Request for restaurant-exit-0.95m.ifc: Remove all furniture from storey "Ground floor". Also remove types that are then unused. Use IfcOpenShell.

First a look at what the model holds.

```python
import ifcopenshell
import ifcopenshell.util.element

model = ifcopenshell.open("restaurant-exit-0.95m.ifc")
print(model.schema)
storey = next(s for s in model.by_type("IfcBuildingStorey") if s.Name == "Ground floor")
furniture = [e for e in ifcopenshell.util.element.get_decomposition(storey) if e.is_a("IfcFurnishingElement")]
seen = {}
for e in furniture:
    element_type = ifcopenshell.util.element.get_type(e)
    name = element_type.Name if element_type not in (None, e) else None
    seen[name] = seen.get(name, 0) + 1
for name, count in sorted(seen.items(), key=str):
    print(count, "x", name)
```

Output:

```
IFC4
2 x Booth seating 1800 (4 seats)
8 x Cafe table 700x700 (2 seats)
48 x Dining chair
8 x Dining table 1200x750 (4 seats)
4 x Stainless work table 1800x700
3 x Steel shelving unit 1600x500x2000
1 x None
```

```python
import ifcopenshell
import ifcopenshell.api.root
import ifcopenshell.util.element

model = ifcopenshell.open("restaurant-exit-0.95m.ifc")

storey = next(s for s in model.by_type("IfcBuildingStorey") if s.Name == "Ground floor")
furniture = [e for e in ifcopenshell.util.element.get_decomposition(storey) if e.is_a("IfcFurnishingElement")]
types = {ifcopenshell.util.element.get_type(e) for e in furniture} - {None, *furniture}

for e in furniture:
    ifcopenshell.api.root.remove_product(model, product=e)
print(len(furniture), "removed")

unused = [t for t in types if not ifcopenshell.util.element.get_types(t)]
for t in unused:
    ifcopenshell.api.root.remove_product(model, product=t)
print(len(unused), "unused types removed")

model.write("restaurant-exit-0.95m_edited.ifc")
```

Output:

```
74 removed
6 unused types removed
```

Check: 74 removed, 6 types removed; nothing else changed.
